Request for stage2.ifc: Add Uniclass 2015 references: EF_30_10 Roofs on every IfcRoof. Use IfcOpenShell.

First a look at what the model holds.

```python
import ifcopenshell

model = ifcopenshell.open("stage2.ifc")
print(model.schema)
print("classifications:", [c.Name for c in model.by_type("IfcClassification")])
for ifc_class in ("IfcDoor", "IfcRoof", "IfcStair", "IfcWall", "IfcWindow"):
    print(ifc_class, len(model.by_type(ifc_class)))
```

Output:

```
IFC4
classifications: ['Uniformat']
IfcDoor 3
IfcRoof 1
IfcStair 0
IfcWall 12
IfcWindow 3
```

```python
import ifcopenshell
import ifcopenshell.api.classification

model = ifcopenshell.open("stage2.ifc")

system = ifcopenshell.api.classification.add_classification(model, classification="Uniclass 2015")

codes = {
    "IfcRoof": ("EF_30_10", "Roofs"),
}
for ifc_class, (code, name) in codes.items():
    products = model.by_type(ifc_class)
    ifcopenshell.api.classification.add_reference(
        model, products=products, classification=system, identification=code, name=name
    )
    print(code, len(products))

model.write("stage2_v2.ifc")
```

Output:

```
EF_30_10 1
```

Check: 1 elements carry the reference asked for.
